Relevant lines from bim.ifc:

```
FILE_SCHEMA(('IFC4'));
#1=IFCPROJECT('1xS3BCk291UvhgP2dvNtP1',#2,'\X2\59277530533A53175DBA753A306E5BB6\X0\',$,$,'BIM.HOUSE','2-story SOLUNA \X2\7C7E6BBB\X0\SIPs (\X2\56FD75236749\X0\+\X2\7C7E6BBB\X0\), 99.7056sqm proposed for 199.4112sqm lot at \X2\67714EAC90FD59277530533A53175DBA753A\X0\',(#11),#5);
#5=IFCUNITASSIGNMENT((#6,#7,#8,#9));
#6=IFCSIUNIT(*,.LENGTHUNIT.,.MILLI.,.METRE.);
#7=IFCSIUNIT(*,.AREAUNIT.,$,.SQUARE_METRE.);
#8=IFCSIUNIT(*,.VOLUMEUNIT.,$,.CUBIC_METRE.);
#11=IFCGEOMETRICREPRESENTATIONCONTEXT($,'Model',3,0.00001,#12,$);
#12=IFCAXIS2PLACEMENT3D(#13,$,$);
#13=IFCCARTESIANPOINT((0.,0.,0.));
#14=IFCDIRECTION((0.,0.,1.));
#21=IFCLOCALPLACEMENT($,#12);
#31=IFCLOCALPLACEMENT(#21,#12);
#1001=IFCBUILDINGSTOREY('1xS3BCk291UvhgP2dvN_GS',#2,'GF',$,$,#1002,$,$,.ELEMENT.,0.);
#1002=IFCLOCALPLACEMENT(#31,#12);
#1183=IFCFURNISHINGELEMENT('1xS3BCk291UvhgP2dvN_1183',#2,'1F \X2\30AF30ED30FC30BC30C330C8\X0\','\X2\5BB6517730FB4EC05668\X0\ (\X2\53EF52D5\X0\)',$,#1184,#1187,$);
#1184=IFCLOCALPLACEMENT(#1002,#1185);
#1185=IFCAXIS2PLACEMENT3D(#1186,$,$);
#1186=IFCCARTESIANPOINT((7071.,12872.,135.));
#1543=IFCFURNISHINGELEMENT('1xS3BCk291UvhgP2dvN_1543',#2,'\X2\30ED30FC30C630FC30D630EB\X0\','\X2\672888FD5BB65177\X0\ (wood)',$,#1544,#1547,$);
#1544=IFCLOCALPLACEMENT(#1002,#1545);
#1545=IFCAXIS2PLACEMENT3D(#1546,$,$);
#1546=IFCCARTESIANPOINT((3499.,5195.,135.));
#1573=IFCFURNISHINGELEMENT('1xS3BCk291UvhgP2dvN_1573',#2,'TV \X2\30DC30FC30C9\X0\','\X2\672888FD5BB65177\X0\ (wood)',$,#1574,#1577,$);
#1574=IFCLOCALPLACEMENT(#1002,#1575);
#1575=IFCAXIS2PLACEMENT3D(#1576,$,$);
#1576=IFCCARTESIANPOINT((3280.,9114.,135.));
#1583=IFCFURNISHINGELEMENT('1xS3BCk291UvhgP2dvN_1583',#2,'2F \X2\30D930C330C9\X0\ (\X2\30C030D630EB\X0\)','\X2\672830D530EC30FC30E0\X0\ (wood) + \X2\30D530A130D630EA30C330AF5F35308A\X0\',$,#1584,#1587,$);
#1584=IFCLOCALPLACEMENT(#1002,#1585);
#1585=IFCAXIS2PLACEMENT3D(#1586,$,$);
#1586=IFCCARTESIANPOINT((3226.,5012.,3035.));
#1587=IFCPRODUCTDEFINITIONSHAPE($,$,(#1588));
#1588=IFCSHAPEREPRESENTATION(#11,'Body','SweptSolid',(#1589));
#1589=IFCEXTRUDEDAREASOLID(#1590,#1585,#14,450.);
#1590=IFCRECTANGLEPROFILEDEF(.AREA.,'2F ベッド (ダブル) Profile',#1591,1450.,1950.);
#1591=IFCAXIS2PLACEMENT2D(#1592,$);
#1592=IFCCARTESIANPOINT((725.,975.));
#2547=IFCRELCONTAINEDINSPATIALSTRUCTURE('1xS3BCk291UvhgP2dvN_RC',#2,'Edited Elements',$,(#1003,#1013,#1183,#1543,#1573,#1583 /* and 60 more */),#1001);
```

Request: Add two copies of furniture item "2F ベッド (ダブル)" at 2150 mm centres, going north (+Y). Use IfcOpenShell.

```python
import numpy as np
import ifcopenshell
import ifcopenshell.api.geometry
import ifcopenshell.api.root
import ifcopenshell.util.element
import ifcopenshell.util.placement

model = ifcopenshell.open("bim.ifc")


def reuse_history(source, copy):
    """copy_class also copies each property set's owner history, people and application; keep the originals."""
    for rel in copy.IsDefinedBy:
        if rel.is_a("IfcRelDefinesByProperties") and (history := rel.RelatingPropertyDefinition.OwnerHistory):
            rel.RelatingPropertyDefinition.OwnerHistory = source.OwnerHistory
            ifcopenshell.util.element.remove_deep2(model, history)


source = model.by_guid("1xS3BCk291UvhgP2dvN_1583")
base = ifcopenshell.util.placement.get_local_placement(source.ObjectPlacement)
step = np.array([0.0, 1.0, 0.0]) * 2150.0

for i in range(1, 3):
    copy = ifcopenshell.api.root.copy_class(model, product=source)
    copy.Representation = ifcopenshell.util.element.copy_deep(
        model, source.Representation, exclude=["IfcGeometricRepresentationContext", "IfcRepresentationMap"]
    )
    reuse_history(source, copy)
    matrix = base.copy()
    matrix[:3, 3] += i * step
    print("added at", matrix[:3, 3].round(3) + 0.0)
    ifcopenshell.api.geometry.edit_object_placement(model, product=copy, matrix=matrix, is_si=False)

model.write("bim-out.ifc")
```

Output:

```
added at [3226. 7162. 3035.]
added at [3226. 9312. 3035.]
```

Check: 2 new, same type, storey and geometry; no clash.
